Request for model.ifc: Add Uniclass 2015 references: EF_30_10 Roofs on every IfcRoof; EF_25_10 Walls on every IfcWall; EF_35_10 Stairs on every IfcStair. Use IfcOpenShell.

First a look at what the model holds.

```python
import ifcopenshell

model = ifcopenshell.open("model.ifc")
print(model.schema)
print("classifications:", [c.Name for c in model.by_type("IfcClassification")])
for ifc_class in ("IfcDoor", "IfcRoof", "IfcStair", "IfcWall", "IfcWindow"):
    print(ifc_class, len(model.by_type(ifc_class)))
```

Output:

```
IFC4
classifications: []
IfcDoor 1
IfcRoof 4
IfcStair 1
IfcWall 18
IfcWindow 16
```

```python
import ifcopenshell
import ifcopenshell.api.classification

model = ifcopenshell.open("model.ifc")

system = ifcopenshell.api.classification.add_classification(model, classification="Uniclass 2015")

codes = {
    "IfcRoof": ("EF_30_10", "Roofs"),
    "IfcWall": ("EF_25_10", "Walls"),
    "IfcStair": ("EF_35_10", "Stairs"),
}
for ifc_class, (code, name) in codes.items():
    products = model.by_type(ifc_class)
    ifcopenshell.api.classification.add_reference(
        model, products=products, classification=system, identification=code, name=name
    )
    print(code, len(products))

model.write("model-out.ifc")
```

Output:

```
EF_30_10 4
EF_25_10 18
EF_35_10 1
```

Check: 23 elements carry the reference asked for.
